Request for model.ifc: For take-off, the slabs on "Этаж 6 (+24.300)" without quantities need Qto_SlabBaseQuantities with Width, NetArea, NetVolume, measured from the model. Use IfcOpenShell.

First a look at what the model holds.

```python
import ifcopenshell
import ifcopenshell.util.element
import ifcopenshell.util.unit

model = ifcopenshell.open("model.ifc")
print(model.schema)
for unit_type in ("LENGTHUNIT", "AREAUNIT", "VOLUMEUNIT"):
    print(unit_type, ifcopenshell.util.unit.calculate_unit_scale(model, unit_type))
storey = next(s for s in model.by_type("IfcBuildingStorey") if s.Name == "Этаж 6 (+24.300)")
slabs = [e for e in ifcopenshell.util.element.get_decomposition(storey) if e.is_a("IfcSlab")]
for e in sorted(slabs, key=lambda e: e.id()):
    print(e.id(), e.is_a(), e.Name, list(ifcopenshell.util.element.get_psets(e, qtos_only=True)), sep=" | ")
```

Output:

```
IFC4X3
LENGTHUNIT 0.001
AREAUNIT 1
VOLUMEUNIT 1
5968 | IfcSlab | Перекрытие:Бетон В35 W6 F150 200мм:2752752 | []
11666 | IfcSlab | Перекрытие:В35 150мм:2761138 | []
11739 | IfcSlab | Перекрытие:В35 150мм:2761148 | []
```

```python
import ifcopenshell
import ifcopenshell.api.pset
import ifcopenshell.geom
import ifcopenshell.util.element
import ifcopenshell.util.shape
import ifcopenshell.util.unit

model = ifcopenshell.open("model.ifc")
unit_scale = ifcopenshell.util.unit.calculate_unit_scale(model)
area_scale = ifcopenshell.util.unit.calculate_unit_scale(model, "AREAUNIT")
volume_scale = ifcopenshell.util.unit.calculate_unit_scale(model, "VOLUMEUNIT")
settings = ifcopenshell.geom.settings()

storey = next(s for s in model.by_type("IfcBuildingStorey") if s.Name == "Этаж 6 (+24.300)")
slabs = [e for e in ifcopenshell.util.element.get_decomposition(storey) if e.is_a("IfcSlab")]

for e in sorted(slabs, key=lambda e: e.id()):
    if ifcopenshell.util.element.get_psets(e, qtos_only=True, should_inherit=False):
        continue
    # Geometry comes back in metres, in the element's own axes.
    shape = ifcopenshell.geom.create_shape(settings, e)
    values = {
        "Width": ifcopenshell.util.shape.get_z(shape.geometry) / unit_scale,
        "NetArea": ifcopenshell.util.shape.get_footprint_area(shape.geometry) / area_scale,
        "NetVolume": ifcopenshell.util.shape.get_volume(shape.geometry) / volume_scale,
    }
    qto = ifcopenshell.api.pset.add_qto(model, product=e, name="Qto_SlabBaseQuantities")
    ifcopenshell.api.pset.edit_qto(model, qto=qto, properties=values)
    print(e.id(), {k: round(v, 3) for k, v in values.items()})

model.write("model_rev.ifc")
```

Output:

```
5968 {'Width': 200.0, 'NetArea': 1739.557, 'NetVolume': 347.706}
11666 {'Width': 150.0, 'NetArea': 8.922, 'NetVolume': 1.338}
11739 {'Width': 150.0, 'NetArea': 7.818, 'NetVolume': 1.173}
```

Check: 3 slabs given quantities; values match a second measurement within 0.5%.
